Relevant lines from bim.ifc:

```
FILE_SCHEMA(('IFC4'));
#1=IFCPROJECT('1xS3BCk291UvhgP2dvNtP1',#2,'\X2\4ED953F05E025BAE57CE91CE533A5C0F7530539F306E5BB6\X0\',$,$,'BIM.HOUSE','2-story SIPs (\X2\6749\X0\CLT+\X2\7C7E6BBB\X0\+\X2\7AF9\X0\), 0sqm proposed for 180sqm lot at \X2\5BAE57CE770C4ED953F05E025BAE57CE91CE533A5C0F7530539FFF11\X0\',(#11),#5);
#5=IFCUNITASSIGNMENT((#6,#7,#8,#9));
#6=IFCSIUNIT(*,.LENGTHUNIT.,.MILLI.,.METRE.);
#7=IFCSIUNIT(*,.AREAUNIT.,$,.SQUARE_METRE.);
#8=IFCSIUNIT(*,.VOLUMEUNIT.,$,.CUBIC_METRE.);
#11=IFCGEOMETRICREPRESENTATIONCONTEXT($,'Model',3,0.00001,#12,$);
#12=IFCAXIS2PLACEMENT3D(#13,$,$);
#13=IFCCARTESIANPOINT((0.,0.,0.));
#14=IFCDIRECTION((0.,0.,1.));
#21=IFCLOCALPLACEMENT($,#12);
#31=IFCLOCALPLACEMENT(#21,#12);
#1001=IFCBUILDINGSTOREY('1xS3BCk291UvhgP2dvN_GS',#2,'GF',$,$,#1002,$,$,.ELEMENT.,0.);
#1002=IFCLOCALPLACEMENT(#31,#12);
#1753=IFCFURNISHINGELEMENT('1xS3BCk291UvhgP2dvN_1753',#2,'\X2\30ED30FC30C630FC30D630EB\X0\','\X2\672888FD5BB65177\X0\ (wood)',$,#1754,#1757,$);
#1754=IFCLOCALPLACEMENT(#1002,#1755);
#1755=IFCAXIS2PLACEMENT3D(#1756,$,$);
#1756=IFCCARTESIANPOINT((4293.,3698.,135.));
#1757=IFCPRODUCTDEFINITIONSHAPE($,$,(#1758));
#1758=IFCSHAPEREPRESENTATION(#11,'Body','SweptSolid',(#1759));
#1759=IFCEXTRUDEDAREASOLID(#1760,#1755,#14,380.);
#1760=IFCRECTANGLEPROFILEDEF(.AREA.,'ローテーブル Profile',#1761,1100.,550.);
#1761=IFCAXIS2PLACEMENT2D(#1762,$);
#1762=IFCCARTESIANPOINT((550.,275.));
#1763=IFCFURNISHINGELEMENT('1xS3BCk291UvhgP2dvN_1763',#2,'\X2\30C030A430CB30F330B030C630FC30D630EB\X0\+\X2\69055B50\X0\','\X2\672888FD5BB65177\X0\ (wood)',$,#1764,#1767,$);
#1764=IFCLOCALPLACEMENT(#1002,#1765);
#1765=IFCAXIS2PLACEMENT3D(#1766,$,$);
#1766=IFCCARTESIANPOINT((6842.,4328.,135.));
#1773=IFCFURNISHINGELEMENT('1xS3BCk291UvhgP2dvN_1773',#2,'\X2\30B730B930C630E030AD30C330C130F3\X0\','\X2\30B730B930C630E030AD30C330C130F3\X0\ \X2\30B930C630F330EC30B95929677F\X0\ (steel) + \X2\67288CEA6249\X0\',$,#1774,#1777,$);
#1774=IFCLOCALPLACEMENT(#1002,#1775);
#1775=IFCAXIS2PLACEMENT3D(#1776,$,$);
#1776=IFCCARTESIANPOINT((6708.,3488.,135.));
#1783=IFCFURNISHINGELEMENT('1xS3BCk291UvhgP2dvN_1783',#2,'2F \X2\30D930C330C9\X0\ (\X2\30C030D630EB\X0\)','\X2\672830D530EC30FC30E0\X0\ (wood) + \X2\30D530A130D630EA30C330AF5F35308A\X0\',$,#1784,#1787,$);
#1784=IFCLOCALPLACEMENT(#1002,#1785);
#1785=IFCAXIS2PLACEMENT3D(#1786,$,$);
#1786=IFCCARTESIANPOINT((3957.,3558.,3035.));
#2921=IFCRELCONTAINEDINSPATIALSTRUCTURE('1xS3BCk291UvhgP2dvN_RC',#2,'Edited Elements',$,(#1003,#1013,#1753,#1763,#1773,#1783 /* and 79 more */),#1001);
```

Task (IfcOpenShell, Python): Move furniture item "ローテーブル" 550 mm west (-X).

```python
import ifcopenshell
import ifcopenshell.api.geometry
import ifcopenshell.util.placement

model = ifcopenshell.open("bim.ifc")

item = model.by_id(1753)
matrix = ifcopenshell.util.placement.get_local_placement(item.ObjectPlacement)
matrix[0, 3] -= 550.0
ifcopenshell.api.geometry.edit_object_placement(model, product=item, matrix=matrix, is_si=False)

print(ifcopenshell.util.placement.get_local_placement(item.ObjectPlacement).round(3) + 0.0)

model.write("bim-out.ifc")
```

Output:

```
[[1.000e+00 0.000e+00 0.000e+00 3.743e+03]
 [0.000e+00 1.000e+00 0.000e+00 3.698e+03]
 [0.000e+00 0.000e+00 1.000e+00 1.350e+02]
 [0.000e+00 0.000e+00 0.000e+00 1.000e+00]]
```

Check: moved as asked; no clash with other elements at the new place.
